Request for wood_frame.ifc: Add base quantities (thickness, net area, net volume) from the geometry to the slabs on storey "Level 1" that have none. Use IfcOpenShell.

First a look at what the model holds.

```python
import ifcopenshell
import ifcopenshell.util.element
import ifcopenshell.util.unit

model = ifcopenshell.open("wood_frame.ifc")
print(model.schema)
for unit_type in ("LENGTHUNIT", "AREAUNIT", "VOLUMEUNIT"):
    print(unit_type, ifcopenshell.util.unit.calculate_unit_scale(model, unit_type))
storey = next(s for s in model.by_type("IfcBuildingStorey") if s.Name == "Level 1")
slabs = [e for e in ifcopenshell.util.element.get_decomposition(storey) if e.is_a("IfcSlab")]
for e in sorted(slabs, key=lambda e: e.id()):
    print(e.id(), e.is_a(), e.Name, list(ifcopenshell.util.element.get_psets(e, qtos_only=True)), sep=" | ")
```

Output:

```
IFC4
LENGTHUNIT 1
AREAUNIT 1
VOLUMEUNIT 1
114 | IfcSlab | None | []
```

```python
import ifcopenshell
import ifcopenshell.api.pset
import ifcopenshell.geom
import ifcopenshell.util.element
import ifcopenshell.util.shape
import ifcopenshell.util.unit

model = ifcopenshell.open("wood_frame.ifc")
unit_scale = ifcopenshell.util.unit.calculate_unit_scale(model)
area_scale = ifcopenshell.util.unit.calculate_unit_scale(model, "AREAUNIT")
volume_scale = ifcopenshell.util.unit.calculate_unit_scale(model, "VOLUMEUNIT")
settings = ifcopenshell.geom.settings()

storey = next(s for s in model.by_type("IfcBuildingStorey") if s.Name == "Level 1")
slabs = [e for e in ifcopenshell.util.element.get_decomposition(storey) if e.is_a("IfcSlab")]

for e in sorted(slabs, key=lambda e: e.id()):
    if ifcopenshell.util.element.get_psets(e, qtos_only=True, should_inherit=False):
        continue
    # Geometry comes back in metres, in the element's own axes.
    shape = ifcopenshell.geom.create_shape(settings, e)
    values = {
        "Width": ifcopenshell.util.shape.get_z(shape.geometry) / unit_scale,
        "NetArea": ifcopenshell.util.shape.get_footprint_area(shape.geometry) / area_scale,
        "NetVolume": ifcopenshell.util.shape.get_volume(shape.geometry) / volume_scale,
    }
    qto = ifcopenshell.api.pset.add_qto(model, product=e, name="Qto_SlabBaseQuantities")
    ifcopenshell.api.pset.edit_qto(model, qto=qto, properties=values)
    print(e.id(), {k: round(v, 3) for k, v in values.items()})

model.write("wood_frame-out.ifc")
```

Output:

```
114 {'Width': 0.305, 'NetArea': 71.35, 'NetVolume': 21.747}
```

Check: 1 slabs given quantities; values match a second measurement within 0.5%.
